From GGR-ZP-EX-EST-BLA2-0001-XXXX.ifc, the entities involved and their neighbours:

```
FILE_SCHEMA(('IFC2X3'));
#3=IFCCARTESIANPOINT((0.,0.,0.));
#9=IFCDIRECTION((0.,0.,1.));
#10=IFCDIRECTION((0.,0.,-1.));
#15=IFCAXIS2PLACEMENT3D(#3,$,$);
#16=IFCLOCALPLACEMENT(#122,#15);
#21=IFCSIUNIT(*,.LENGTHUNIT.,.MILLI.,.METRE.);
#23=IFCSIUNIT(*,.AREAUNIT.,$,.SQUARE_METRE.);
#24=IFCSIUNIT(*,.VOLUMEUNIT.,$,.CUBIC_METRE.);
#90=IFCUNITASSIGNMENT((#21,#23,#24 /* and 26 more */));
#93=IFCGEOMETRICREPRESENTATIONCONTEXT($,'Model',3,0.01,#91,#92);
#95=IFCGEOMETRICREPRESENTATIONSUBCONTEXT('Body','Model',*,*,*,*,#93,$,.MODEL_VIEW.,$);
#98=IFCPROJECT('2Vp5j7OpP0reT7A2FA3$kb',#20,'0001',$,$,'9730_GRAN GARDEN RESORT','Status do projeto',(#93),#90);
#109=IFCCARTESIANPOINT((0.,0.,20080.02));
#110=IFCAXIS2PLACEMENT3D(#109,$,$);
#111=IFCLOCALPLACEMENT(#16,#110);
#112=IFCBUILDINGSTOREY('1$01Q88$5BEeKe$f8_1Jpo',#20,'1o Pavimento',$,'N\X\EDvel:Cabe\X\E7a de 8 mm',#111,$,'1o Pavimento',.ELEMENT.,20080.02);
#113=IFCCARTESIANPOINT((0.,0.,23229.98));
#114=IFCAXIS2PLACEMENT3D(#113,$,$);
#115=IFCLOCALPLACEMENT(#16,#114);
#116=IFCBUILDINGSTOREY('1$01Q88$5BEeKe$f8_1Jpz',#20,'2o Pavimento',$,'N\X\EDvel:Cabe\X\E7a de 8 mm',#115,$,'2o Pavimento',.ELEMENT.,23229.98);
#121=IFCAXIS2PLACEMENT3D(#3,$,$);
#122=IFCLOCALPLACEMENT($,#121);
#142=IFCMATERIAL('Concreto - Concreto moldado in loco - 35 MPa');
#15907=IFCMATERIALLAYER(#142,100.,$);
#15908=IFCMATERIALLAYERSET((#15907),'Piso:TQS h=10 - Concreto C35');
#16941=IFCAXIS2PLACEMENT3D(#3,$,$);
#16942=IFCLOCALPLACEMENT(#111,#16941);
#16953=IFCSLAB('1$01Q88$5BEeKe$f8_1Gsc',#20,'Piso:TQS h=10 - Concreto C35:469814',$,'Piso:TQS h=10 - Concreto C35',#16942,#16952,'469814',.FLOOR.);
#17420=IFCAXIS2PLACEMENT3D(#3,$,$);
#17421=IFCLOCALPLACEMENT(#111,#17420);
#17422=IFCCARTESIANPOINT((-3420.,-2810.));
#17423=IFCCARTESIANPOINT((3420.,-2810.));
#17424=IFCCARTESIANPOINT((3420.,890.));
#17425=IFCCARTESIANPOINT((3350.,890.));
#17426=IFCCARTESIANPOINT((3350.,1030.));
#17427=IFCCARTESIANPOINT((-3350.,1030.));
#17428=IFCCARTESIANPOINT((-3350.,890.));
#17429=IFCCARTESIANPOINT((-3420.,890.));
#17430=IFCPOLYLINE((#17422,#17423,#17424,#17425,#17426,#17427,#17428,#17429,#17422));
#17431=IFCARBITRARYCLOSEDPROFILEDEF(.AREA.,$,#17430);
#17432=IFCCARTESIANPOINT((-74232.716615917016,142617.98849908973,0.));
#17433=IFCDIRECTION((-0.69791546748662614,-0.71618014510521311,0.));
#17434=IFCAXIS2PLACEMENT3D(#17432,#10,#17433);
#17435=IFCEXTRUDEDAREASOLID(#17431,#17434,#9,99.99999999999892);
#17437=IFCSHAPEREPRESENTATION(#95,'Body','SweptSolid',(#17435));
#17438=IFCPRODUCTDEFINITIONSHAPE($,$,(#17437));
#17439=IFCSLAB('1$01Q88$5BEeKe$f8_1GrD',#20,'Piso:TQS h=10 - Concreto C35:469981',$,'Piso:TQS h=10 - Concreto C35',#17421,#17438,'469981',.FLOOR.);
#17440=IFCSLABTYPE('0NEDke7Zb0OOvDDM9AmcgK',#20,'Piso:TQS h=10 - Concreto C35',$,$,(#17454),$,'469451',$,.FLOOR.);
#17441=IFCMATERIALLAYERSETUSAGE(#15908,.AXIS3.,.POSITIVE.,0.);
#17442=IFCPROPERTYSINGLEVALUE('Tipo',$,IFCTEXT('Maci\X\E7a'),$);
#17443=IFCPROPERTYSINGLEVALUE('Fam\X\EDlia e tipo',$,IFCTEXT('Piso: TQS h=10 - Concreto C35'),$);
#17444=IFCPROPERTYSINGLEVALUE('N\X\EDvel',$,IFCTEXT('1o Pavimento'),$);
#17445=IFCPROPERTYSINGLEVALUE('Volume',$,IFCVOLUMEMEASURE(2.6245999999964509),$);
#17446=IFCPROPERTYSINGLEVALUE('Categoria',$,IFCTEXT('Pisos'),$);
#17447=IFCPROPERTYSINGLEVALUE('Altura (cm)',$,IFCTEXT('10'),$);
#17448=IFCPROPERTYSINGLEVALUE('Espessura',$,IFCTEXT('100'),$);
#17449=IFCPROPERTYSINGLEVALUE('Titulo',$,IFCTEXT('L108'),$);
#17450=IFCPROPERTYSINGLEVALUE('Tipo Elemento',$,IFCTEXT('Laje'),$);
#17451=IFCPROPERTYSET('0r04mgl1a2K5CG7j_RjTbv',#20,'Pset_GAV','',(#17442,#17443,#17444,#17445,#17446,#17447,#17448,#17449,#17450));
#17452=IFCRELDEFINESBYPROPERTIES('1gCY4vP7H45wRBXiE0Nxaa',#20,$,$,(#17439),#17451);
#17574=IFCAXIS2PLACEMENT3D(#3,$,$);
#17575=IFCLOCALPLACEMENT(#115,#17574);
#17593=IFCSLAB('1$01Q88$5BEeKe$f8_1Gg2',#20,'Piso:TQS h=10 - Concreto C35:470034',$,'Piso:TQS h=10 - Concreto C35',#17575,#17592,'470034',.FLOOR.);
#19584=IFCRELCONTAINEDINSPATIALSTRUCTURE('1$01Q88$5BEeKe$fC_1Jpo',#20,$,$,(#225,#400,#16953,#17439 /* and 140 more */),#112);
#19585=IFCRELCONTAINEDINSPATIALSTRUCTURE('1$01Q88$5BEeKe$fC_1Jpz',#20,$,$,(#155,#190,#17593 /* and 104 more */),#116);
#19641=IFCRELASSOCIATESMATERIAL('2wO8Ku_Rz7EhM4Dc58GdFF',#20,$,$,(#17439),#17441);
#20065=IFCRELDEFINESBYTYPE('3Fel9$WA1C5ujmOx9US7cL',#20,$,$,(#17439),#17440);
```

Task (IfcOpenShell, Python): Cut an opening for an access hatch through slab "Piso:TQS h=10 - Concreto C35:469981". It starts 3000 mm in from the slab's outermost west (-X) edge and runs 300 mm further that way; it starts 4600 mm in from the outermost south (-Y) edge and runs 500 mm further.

```python
import numpy as np
import ifcopenshell
import ifcopenshell.api.feature
import ifcopenshell.api.geometry
import ifcopenshell.api.pset
import ifcopenshell.api.root
import ifcopenshell.geom
import ifcopenshell.util.element
import ifcopenshell.util.placement
import ifcopenshell.util.representation
import ifcopenshell.util.shape
import ifcopenshell.util.unit

model = ifcopenshell.open("GGR-ZP-EX-EST-BLA2-0001-XXXX.ifc")
unit_scale = ifcopenshell.util.unit.calculate_unit_scale(model)
volume_scale = ifcopenshell.util.unit.calculate_unit_scale(model, "VOLUMEUNIT")
settings = ifcopenshell.geom.settings()


def volume(element):
    """Net volume in cubic metres, openings subtracted."""
    shape = ifcopenshell.geom.create_shape(settings, element)
    return ifcopenshell.util.shape.get_volume(shape.geometry)


slab = model.by_id(17439)
before = volume(slab)

# Extent in the slab's own axes, in metres. The edges named are its -X and -Y sides.
slab_shape = ifcopenshell.geom.create_shape(settings, slab)
vertices = ifcopenshell.util.shape.get_vertices(slab_shape.geometry)
x_min, y_min, bottom = vertices.min(axis=0)
top = vertices[:, 2].max()

opening = ifcopenshell.api.root.create_entity(model, ifc_class="IfcOpeningElement", name="Access hatch opening")
context = ifcopenshell.util.representation.get_context(model, "Model", "Body", "MODEL_VIEW")
width, depth = 0.3, 0.5
outline = [(0.0, 0.0), (width, 0.0), (width, depth), (0.0, depth), (0.0, 0.0)]
# Overshoot both faces by 50 mm so the cut is clean.
shape = ifcopenshell.api.geometry.add_slab_representation(
    model, context=context, depth=top - bottom + 0.1, polyline=outline
)
ifcopenshell.api.geometry.assign_representation(model, product=opening, representation=shape)

matrix = ifcopenshell.util.placement.get_local_placement(slab.ObjectPlacement)
matrix[:, 3] = matrix @ np.append(np.array([x_min + 3, y_min + 4.6, bottom - 0.05]) / unit_scale, 1.0)
ifcopenshell.api.geometry.edit_object_placement(model, product=opening, matrix=matrix, is_si=False)
ifcopenshell.api.feature.add_feature(model, feature=opening, element=slab)

after = volume(slab)

# Update the slab's stored quantities.
pset = model.by_id(ifcopenshell.util.element.get_pset(slab, "Pset_GAV", should_inherit=False)["id"])
ifcopenshell.api.pset.edit_pset(model, pset=pset, properties={
    "Volume": model.create_entity("IfcVolumeMeasure", after / volume_scale),
})

print(f"slab volume {before:.3f} -> {after:.3f} m3")

model.write("GGR-ZP-EX-EST-BLA2-0001-XXXX_updated.ifc")
```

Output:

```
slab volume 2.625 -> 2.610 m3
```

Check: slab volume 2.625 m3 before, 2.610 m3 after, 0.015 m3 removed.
